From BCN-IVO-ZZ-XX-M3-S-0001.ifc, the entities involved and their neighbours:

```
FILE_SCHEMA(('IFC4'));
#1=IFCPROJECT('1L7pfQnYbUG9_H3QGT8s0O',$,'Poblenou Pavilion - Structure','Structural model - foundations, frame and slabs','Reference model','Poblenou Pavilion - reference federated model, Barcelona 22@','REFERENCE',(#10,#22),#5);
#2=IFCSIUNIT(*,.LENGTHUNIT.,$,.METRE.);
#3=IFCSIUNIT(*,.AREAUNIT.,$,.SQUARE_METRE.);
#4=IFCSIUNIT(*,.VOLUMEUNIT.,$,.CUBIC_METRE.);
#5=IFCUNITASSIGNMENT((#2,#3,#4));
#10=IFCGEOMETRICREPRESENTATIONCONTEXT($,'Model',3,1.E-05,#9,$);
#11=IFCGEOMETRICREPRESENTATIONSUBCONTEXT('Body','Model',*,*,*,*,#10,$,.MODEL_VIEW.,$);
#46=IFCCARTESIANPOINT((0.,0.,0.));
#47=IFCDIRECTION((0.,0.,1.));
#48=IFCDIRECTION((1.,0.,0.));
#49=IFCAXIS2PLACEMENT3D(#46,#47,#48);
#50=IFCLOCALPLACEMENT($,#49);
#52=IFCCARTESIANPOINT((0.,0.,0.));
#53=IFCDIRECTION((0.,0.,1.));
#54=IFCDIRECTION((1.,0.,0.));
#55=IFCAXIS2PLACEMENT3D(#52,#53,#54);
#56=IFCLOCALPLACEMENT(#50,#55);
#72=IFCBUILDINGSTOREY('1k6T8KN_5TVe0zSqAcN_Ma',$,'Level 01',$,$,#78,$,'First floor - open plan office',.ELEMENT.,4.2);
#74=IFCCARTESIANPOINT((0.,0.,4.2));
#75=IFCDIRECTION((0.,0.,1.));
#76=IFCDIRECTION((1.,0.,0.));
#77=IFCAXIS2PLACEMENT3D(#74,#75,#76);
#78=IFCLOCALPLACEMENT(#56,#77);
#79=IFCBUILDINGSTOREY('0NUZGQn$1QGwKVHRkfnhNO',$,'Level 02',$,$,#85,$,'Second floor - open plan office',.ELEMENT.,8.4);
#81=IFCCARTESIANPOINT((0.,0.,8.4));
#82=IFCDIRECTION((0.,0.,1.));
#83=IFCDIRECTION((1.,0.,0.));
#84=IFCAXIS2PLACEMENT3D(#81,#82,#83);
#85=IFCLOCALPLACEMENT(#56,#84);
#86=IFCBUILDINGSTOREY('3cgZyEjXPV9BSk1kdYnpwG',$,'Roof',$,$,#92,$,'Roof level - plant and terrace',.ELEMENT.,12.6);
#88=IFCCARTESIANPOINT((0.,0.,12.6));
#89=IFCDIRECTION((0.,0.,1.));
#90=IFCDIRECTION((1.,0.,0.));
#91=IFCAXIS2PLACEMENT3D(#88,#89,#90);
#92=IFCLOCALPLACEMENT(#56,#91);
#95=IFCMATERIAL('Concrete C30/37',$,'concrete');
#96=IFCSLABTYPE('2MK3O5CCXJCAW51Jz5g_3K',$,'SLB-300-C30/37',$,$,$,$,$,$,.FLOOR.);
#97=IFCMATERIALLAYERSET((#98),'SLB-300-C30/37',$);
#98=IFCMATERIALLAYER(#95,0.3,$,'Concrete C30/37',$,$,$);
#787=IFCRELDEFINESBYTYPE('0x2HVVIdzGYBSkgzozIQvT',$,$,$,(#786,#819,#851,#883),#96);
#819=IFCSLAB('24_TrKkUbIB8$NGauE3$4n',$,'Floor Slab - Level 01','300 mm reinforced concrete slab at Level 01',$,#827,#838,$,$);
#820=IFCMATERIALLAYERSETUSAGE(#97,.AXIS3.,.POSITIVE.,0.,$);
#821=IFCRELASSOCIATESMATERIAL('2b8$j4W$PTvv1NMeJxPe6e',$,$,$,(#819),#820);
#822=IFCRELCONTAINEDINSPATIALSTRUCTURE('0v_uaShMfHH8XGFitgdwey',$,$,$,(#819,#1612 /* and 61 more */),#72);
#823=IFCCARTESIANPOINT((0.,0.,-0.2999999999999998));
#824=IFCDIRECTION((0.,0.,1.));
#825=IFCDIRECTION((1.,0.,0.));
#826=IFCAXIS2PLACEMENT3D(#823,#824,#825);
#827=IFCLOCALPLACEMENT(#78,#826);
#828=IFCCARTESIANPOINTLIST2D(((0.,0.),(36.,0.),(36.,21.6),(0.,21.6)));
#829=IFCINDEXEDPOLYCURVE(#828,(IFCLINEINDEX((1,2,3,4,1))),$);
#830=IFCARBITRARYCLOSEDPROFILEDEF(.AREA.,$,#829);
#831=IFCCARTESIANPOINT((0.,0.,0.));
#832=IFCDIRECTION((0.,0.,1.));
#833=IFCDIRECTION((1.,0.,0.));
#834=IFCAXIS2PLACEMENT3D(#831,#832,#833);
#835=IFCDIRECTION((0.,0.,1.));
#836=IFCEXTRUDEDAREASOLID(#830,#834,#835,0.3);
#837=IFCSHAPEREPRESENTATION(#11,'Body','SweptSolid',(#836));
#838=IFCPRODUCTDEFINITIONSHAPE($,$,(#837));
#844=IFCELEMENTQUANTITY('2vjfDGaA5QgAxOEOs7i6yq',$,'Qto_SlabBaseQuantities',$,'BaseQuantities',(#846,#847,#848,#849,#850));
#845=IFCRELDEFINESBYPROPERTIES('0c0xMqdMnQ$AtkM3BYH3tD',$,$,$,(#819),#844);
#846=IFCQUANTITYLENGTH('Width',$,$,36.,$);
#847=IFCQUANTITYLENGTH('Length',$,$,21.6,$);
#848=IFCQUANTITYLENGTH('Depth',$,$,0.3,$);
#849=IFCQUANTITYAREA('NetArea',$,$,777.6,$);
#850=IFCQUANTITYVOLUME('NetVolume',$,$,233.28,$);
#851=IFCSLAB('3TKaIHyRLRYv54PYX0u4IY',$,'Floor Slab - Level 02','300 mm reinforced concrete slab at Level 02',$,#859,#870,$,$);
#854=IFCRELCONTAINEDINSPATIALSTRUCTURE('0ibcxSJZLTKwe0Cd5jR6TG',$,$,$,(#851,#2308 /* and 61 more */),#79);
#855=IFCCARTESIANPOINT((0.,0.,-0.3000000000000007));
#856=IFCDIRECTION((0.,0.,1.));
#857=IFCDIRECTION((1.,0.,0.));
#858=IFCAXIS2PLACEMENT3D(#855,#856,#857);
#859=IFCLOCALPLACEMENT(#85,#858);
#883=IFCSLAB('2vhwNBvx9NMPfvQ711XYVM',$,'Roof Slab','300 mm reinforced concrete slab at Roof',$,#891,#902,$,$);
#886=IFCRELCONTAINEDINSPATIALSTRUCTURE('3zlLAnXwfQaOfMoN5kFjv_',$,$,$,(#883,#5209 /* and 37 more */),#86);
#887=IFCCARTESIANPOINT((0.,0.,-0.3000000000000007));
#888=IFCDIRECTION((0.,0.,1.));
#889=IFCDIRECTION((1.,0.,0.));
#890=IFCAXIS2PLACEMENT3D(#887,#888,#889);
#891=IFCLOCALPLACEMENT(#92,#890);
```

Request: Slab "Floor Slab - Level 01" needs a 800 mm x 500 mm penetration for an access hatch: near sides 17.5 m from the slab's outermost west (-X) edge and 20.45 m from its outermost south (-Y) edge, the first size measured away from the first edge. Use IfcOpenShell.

```python
import numpy as np
import ifcopenshell
import ifcopenshell.api.feature
import ifcopenshell.api.geometry
import ifcopenshell.api.pset
import ifcopenshell.api.root
import ifcopenshell.geom
import ifcopenshell.util.element
import ifcopenshell.util.placement
import ifcopenshell.util.representation
import ifcopenshell.util.shape
import ifcopenshell.util.unit

model = ifcopenshell.open("BCN-IVO-ZZ-XX-M3-S-0001.ifc")
unit_scale = ifcopenshell.util.unit.calculate_unit_scale(model)
area_scale = ifcopenshell.util.unit.calculate_unit_scale(model, "AREAUNIT")
volume_scale = ifcopenshell.util.unit.calculate_unit_scale(model, "VOLUMEUNIT")
settings = ifcopenshell.geom.settings()


def volume(element):
    """Net volume in cubic metres, openings subtracted."""
    shape = ifcopenshell.geom.create_shape(settings, element)
    return ifcopenshell.util.shape.get_volume(shape.geometry)


slab = model.by_guid("24_TrKkUbIB8$NGauE3$4n")
before = volume(slab)

# Extent in the slab's own axes, in metres. The edges named are its -X and -Y sides.
slab_shape = ifcopenshell.geom.create_shape(settings, slab)
vertices = ifcopenshell.util.shape.get_vertices(slab_shape.geometry)
x_min, y_min, bottom = vertices.min(axis=0)
top = vertices[:, 2].max()

opening = ifcopenshell.api.root.create_entity(model, ifc_class="IfcOpeningElement", name="Access hatch opening", predefined_type="OPENING")
context = ifcopenshell.util.representation.get_context(model, "Model", "Body", "MODEL_VIEW")
width, depth = 0.8, 0.5
outline = [(0.0, 0.0), (width, 0.0), (width, depth), (0.0, depth), (0.0, 0.0)]
# Overshoot both faces by 50 mm so the cut is clean.
shape = ifcopenshell.api.geometry.add_slab_representation(
    model, context=context, depth=top - bottom + 0.1, polyline=outline
)
ifcopenshell.api.geometry.assign_representation(model, product=opening, representation=shape)

matrix = ifcopenshell.util.placement.get_local_placement(slab.ObjectPlacement)
matrix[:, 3] = matrix @ np.append(np.array([x_min + 17.5, y_min + 20.45, bottom - 0.05]) / unit_scale, 1.0)
ifcopenshell.api.geometry.edit_object_placement(model, product=opening, matrix=matrix, is_si=False)
ifcopenshell.api.feature.add_feature(model, feature=opening, element=slab)

after = volume(slab)

# Update the slab's stored quantities.
qto = model.by_id(ifcopenshell.util.element.get_pset(slab, "Qto_SlabBaseQuantities", should_inherit=False)["id"])
ifcopenshell.api.pset.edit_qto(model, qto=qto, properties={
    "NetArea": after / (top - bottom) / area_scale,
    "NetVolume": after / volume_scale,
})

print(f"slab volume {before:.3f} -> {after:.3f} m3")

model.write("BCN-IVO-ZZ-XX-M3-S-0001-out.ifc")
```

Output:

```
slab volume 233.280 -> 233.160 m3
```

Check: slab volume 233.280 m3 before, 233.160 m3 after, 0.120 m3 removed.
